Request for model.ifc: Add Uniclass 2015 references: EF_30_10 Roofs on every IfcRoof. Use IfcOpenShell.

First a look at what the model holds.

```python
import ifcopenshell

model = ifcopenshell.open("model.ifc")
print(model.schema)
print("classifications:", [c.Name for c in model.by_type("IfcClassification")])
for ifc_class in ("IfcDoor", "IfcRoof", "IfcStair", "IfcWall", "IfcWindow"):
    print(ifc_class, len(model.by_type(ifc_class)))
```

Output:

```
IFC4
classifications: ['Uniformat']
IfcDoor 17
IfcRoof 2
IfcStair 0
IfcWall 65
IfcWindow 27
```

```python
import ifcopenshell
import ifcopenshell.api.classification

model = ifcopenshell.open("model.ifc")

system = ifcopenshell.api.classification.add_classification(model, classification="Uniclass 2015")

codes = {
    "IfcRoof": ("EF_30_10", "Roofs"),
}
for ifc_class, (code, name) in codes.items():
    products = model.by_type(ifc_class)
    ifcopenshell.api.classification.add_reference(
        model, products=products, classification=system, identification=code, name=name
    )
    print(code, len(products))

model.write("model-out.ifc")
```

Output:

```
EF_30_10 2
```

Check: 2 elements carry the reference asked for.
